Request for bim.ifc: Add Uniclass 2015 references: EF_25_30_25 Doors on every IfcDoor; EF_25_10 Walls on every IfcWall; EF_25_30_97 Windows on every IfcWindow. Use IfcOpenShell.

First a look at what the model holds.

```python
import ifcopenshell

model = ifcopenshell.open("bim.ifc")
print(model.schema)
print("classifications:", [c.Name for c in model.by_type("IfcClassification")])
for ifc_class in ("IfcDoor", "IfcRoof", "IfcStair", "IfcWall", "IfcWindow"):
    print(ifc_class, len(model.by_type(ifc_class)))
```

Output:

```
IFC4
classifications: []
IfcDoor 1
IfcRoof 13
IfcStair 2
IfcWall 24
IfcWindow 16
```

```python
import ifcopenshell
import ifcopenshell.api.classification

model = ifcopenshell.open("bim.ifc")

system = ifcopenshell.api.classification.add_classification(model, classification="Uniclass 2015")

codes = {
    "IfcDoor": ("EF_25_30_25", "Doors"),
    "IfcWall": ("EF_25_10", "Walls"),
    "IfcWindow": ("EF_25_30_97", "Windows"),
}
for ifc_class, (code, name) in codes.items():
    products = model.by_type(ifc_class)
    ifcopenshell.api.classification.add_reference(
        model, products=products, classification=system, identification=code, name=name
    )
    print(code, len(products))

model.write("bim_rev.ifc")
```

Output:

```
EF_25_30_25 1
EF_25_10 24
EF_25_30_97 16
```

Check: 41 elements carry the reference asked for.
